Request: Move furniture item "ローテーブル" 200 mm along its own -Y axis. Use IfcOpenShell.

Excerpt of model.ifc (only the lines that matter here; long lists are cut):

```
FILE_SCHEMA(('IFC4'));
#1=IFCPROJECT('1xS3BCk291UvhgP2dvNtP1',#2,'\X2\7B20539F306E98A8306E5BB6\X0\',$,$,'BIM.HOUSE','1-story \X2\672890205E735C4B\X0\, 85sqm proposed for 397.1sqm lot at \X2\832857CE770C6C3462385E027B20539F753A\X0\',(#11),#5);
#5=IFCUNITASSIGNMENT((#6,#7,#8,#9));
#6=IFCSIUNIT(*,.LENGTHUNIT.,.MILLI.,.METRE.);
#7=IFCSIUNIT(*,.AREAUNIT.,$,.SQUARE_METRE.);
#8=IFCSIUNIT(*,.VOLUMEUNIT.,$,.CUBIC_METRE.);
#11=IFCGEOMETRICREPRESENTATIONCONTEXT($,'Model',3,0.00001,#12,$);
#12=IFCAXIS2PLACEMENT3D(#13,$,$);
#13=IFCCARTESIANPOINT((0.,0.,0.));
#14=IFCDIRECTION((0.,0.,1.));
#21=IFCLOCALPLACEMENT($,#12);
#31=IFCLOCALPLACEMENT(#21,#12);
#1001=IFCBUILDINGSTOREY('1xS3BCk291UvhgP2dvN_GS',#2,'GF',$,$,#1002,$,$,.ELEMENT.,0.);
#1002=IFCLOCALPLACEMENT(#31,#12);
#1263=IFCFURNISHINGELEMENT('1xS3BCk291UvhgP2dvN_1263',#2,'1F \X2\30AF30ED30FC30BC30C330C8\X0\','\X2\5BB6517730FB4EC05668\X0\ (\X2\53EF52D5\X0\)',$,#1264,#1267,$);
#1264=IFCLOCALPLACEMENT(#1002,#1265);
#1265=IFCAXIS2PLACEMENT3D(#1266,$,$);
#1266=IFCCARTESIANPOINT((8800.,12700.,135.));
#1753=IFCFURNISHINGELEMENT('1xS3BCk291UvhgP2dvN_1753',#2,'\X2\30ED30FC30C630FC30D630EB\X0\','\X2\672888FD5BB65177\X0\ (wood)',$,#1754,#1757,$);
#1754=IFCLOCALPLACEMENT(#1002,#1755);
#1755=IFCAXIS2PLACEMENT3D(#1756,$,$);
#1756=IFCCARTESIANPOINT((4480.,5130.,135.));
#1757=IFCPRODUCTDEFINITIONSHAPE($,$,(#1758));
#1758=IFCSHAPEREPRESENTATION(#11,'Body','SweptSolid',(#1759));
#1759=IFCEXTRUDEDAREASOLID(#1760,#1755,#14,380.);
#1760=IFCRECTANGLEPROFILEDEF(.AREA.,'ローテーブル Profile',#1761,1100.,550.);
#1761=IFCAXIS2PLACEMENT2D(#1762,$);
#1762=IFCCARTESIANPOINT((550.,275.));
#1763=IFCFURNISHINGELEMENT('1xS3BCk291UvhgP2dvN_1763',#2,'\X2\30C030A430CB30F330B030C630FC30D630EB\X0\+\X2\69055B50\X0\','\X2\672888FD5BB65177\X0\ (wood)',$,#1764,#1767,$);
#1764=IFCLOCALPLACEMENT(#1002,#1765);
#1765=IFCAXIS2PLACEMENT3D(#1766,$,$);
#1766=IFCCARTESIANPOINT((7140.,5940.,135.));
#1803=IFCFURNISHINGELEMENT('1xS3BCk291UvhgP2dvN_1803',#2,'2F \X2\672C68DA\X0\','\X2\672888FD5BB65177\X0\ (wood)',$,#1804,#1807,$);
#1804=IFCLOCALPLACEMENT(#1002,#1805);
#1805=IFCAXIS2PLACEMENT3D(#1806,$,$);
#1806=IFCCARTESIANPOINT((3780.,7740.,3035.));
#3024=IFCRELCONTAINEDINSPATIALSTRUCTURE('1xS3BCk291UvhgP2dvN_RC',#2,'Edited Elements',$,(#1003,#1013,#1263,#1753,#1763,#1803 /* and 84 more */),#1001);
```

```python
import ifcopenshell
import ifcopenshell.api.geometry
import ifcopenshell.util.placement
import ifcopenshell.util.unit

model = ifcopenshell.open("model.ifc")
unit_scale = ifcopenshell.util.unit.calculate_unit_scale(model)

item = model.by_id(1753)
matrix = ifcopenshell.util.placement.get_local_placement(item.ObjectPlacement)
matrix[:3, 3] -= matrix[:3, 1] * 0.2 / unit_scale
ifcopenshell.api.geometry.edit_object_placement(model, product=item, matrix=matrix, is_si=False)

print(ifcopenshell.util.placement.get_local_placement(item.ObjectPlacement).round(3) + 0.0)

model.write("model_rev.ifc")
```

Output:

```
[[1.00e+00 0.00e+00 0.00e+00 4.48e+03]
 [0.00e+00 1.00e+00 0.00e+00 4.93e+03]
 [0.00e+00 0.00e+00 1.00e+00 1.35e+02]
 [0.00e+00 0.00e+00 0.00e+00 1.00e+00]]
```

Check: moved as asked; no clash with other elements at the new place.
